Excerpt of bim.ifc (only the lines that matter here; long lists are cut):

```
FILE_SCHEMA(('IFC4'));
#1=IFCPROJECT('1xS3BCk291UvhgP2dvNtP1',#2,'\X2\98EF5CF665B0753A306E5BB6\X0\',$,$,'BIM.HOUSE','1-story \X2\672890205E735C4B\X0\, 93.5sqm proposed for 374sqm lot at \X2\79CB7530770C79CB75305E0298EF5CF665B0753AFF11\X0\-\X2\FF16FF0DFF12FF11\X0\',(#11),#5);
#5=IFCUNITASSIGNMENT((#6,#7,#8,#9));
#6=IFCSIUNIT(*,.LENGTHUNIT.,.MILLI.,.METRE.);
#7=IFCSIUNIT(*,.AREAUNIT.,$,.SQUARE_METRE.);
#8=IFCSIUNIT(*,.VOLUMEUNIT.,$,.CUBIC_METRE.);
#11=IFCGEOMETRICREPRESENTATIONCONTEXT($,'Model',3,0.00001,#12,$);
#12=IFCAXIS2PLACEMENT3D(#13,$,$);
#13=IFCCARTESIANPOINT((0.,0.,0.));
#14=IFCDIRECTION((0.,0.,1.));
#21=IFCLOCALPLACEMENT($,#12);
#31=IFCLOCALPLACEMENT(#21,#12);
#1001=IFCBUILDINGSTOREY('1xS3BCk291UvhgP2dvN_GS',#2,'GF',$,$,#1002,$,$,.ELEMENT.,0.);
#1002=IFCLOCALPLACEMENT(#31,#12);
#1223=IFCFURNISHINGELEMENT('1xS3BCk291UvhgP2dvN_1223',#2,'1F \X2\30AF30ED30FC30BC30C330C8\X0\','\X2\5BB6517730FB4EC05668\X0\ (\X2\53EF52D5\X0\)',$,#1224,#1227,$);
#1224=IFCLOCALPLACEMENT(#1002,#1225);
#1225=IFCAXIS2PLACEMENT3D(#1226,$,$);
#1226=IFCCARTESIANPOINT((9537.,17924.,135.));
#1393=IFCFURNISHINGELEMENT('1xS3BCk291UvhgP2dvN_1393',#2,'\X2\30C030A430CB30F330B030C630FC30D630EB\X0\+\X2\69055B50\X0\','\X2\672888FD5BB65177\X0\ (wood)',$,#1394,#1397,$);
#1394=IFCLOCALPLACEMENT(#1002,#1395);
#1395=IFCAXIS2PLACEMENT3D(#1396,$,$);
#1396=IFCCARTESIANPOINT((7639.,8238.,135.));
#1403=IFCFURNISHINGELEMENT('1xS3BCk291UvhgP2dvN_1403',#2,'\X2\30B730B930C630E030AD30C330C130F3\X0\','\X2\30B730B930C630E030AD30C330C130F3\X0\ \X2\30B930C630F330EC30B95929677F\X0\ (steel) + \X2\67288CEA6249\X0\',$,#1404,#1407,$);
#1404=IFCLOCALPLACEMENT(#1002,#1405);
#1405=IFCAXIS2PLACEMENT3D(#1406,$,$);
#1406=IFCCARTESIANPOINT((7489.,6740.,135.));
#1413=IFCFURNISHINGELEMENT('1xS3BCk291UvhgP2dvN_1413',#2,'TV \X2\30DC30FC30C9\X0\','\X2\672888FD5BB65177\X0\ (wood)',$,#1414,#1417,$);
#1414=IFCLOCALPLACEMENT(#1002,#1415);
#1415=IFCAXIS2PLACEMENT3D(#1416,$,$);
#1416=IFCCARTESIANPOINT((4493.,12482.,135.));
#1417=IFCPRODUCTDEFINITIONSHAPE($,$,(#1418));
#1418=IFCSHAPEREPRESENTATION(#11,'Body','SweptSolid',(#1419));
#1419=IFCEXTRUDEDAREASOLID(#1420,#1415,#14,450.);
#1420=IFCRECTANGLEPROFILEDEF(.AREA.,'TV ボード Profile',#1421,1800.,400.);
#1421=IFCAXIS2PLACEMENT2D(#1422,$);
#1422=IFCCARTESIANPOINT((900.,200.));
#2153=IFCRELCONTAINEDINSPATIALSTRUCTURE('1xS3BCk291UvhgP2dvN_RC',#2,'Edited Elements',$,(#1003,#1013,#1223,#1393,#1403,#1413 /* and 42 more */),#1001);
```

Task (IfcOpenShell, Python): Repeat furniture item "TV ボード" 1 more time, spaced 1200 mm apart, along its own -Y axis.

```python
import ifcopenshell
import ifcopenshell.api.geometry
import ifcopenshell.api.root
import ifcopenshell.util.element
import ifcopenshell.util.placement

model = ifcopenshell.open("bim.ifc")


def reuse_history(source, copy):
    """copy_class also copies each property set's owner history, people and application; keep the originals."""
    for rel in copy.IsDefinedBy:
        if rel.is_a("IfcRelDefinesByProperties") and (history := rel.RelatingPropertyDefinition.OwnerHistory):
            rel.RelatingPropertyDefinition.OwnerHistory = source.OwnerHistory
            ifcopenshell.util.element.remove_deep2(model, history)


source = model.by_id(1413)
base = ifcopenshell.util.placement.get_local_placement(source.ObjectPlacement)
step = -base[:3, 1] * 1200.0

for i in range(1, 2):
    copy = ifcopenshell.api.root.copy_class(model, product=source)
    copy.Representation = ifcopenshell.util.element.copy_deep(
        model, source.Representation, exclude=["IfcGeometricRepresentationContext", "IfcRepresentationMap"]
    )
    reuse_history(source, copy)
    matrix = base.copy()
    matrix[:3, 3] += i * step
    print("added at", matrix[:3, 3].round(3) + 0.0)
    ifcopenshell.api.geometry.edit_object_placement(model, product=copy, matrix=matrix, is_si=False)

model.write("bim_edited.ifc")
```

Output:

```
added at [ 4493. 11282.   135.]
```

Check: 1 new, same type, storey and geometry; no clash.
